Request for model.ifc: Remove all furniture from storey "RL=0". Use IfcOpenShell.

First a look at what the model holds.

```python
import ifcopenshell
import ifcopenshell.util.element

model = ifcopenshell.open("model.ifc")
print(model.schema)
storey = next(s for s in model.by_type("IfcBuildingStorey") if s.Name == "RL=0")
furniture = [e for e in ifcopenshell.util.element.get_decomposition(storey) if e.is_a("IfcFurnishingElement")]
seen = {}
for e in furniture:
    element_type = ifcopenshell.util.element.get_type(e)
    name = element_type.Name if element_type not in (None, e) else None
    seen[name] = seen.get(name, 0) + 1
for name, count in sorted(seen.items(), key=str):
    print(count, "x", name)
```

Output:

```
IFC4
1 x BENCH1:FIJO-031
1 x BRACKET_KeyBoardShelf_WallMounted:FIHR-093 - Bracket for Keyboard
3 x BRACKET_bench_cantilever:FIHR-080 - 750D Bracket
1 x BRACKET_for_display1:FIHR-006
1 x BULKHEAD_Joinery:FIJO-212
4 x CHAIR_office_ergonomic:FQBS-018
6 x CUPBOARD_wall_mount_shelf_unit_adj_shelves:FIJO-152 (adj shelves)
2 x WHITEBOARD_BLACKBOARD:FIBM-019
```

```python
import ifcopenshell
import ifcopenshell.api.root
import ifcopenshell.util.element

model = ifcopenshell.open("model.ifc")

storey = next(s for s in model.by_type("IfcBuildingStorey") if s.Name == "RL=0")
furniture = [e for e in ifcopenshell.util.element.get_decomposition(storey) if e.is_a("IfcFurnishingElement")]

for e in furniture:
    ifcopenshell.api.root.remove_product(model, product=e)
print(len(furniture), "removed")

model.write("model-out.ifc")
```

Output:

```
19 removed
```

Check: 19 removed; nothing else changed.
